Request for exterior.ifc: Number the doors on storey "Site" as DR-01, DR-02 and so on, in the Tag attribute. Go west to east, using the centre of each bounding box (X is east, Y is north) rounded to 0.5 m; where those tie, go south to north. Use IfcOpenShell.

First a look at what the model holds.

```python
import ifcopenshell
import ifcopenshell.util.element
import ifcopenshell.util.placement

model = ifcopenshell.open("exterior.ifc")
print(model.schema)
storey = next(s for s in model.by_type("IfcBuildingStorey") if s.Name == "Site")
doors = [e for e in ifcopenshell.util.element.get_decomposition(storey) if e.is_a("IfcDoor")]
for e in sorted(doors, key=lambda e: e.id()):
    origin = ifcopenshell.util.placement.get_local_placement(e.ObjectPlacement)[:3, 3]
    print(e.id(), e.Tag, e.Name, origin.round(2) + 0.0, sep=" | ")
```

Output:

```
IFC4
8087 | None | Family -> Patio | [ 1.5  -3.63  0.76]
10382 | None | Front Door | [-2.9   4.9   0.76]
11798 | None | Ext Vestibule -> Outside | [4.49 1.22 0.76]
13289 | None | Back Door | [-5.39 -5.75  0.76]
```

```python
import ifcopenshell
import ifcopenshell.geom
import ifcopenshell.util.element
import ifcopenshell.util.shape

model = ifcopenshell.open("exterior.ifc")
settings = ifcopenshell.geom.settings()
settings.set("use-world-coords", True)


def centre(element):
    shape = ifcopenshell.geom.create_shape(settings, element)
    return ifcopenshell.util.shape.get_bbox_centroid(shape.geometry)


storey = next(s for s in model.by_type("IfcBuildingStorey") if s.Name == "Site")
doors = [e for e in ifcopenshell.util.element.get_decomposition(storey) if e.is_a("IfcDoor")]

# Insertion points can sit at a corner or the storey origin, so sort by the geometry (in metres).
centres = {e: centre(e) for e in doors}
doors.sort(key=lambda e: (round(centres[e][0] / 0.5), centres[e][1]))

for i, e in enumerate(doors, start=1):
    number = f"DR-{i:02d}"
    e.Tag = number
    print(e.id(), number)

model.write("exterior_v2.ifc")
```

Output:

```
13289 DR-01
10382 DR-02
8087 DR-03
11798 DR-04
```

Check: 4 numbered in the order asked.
